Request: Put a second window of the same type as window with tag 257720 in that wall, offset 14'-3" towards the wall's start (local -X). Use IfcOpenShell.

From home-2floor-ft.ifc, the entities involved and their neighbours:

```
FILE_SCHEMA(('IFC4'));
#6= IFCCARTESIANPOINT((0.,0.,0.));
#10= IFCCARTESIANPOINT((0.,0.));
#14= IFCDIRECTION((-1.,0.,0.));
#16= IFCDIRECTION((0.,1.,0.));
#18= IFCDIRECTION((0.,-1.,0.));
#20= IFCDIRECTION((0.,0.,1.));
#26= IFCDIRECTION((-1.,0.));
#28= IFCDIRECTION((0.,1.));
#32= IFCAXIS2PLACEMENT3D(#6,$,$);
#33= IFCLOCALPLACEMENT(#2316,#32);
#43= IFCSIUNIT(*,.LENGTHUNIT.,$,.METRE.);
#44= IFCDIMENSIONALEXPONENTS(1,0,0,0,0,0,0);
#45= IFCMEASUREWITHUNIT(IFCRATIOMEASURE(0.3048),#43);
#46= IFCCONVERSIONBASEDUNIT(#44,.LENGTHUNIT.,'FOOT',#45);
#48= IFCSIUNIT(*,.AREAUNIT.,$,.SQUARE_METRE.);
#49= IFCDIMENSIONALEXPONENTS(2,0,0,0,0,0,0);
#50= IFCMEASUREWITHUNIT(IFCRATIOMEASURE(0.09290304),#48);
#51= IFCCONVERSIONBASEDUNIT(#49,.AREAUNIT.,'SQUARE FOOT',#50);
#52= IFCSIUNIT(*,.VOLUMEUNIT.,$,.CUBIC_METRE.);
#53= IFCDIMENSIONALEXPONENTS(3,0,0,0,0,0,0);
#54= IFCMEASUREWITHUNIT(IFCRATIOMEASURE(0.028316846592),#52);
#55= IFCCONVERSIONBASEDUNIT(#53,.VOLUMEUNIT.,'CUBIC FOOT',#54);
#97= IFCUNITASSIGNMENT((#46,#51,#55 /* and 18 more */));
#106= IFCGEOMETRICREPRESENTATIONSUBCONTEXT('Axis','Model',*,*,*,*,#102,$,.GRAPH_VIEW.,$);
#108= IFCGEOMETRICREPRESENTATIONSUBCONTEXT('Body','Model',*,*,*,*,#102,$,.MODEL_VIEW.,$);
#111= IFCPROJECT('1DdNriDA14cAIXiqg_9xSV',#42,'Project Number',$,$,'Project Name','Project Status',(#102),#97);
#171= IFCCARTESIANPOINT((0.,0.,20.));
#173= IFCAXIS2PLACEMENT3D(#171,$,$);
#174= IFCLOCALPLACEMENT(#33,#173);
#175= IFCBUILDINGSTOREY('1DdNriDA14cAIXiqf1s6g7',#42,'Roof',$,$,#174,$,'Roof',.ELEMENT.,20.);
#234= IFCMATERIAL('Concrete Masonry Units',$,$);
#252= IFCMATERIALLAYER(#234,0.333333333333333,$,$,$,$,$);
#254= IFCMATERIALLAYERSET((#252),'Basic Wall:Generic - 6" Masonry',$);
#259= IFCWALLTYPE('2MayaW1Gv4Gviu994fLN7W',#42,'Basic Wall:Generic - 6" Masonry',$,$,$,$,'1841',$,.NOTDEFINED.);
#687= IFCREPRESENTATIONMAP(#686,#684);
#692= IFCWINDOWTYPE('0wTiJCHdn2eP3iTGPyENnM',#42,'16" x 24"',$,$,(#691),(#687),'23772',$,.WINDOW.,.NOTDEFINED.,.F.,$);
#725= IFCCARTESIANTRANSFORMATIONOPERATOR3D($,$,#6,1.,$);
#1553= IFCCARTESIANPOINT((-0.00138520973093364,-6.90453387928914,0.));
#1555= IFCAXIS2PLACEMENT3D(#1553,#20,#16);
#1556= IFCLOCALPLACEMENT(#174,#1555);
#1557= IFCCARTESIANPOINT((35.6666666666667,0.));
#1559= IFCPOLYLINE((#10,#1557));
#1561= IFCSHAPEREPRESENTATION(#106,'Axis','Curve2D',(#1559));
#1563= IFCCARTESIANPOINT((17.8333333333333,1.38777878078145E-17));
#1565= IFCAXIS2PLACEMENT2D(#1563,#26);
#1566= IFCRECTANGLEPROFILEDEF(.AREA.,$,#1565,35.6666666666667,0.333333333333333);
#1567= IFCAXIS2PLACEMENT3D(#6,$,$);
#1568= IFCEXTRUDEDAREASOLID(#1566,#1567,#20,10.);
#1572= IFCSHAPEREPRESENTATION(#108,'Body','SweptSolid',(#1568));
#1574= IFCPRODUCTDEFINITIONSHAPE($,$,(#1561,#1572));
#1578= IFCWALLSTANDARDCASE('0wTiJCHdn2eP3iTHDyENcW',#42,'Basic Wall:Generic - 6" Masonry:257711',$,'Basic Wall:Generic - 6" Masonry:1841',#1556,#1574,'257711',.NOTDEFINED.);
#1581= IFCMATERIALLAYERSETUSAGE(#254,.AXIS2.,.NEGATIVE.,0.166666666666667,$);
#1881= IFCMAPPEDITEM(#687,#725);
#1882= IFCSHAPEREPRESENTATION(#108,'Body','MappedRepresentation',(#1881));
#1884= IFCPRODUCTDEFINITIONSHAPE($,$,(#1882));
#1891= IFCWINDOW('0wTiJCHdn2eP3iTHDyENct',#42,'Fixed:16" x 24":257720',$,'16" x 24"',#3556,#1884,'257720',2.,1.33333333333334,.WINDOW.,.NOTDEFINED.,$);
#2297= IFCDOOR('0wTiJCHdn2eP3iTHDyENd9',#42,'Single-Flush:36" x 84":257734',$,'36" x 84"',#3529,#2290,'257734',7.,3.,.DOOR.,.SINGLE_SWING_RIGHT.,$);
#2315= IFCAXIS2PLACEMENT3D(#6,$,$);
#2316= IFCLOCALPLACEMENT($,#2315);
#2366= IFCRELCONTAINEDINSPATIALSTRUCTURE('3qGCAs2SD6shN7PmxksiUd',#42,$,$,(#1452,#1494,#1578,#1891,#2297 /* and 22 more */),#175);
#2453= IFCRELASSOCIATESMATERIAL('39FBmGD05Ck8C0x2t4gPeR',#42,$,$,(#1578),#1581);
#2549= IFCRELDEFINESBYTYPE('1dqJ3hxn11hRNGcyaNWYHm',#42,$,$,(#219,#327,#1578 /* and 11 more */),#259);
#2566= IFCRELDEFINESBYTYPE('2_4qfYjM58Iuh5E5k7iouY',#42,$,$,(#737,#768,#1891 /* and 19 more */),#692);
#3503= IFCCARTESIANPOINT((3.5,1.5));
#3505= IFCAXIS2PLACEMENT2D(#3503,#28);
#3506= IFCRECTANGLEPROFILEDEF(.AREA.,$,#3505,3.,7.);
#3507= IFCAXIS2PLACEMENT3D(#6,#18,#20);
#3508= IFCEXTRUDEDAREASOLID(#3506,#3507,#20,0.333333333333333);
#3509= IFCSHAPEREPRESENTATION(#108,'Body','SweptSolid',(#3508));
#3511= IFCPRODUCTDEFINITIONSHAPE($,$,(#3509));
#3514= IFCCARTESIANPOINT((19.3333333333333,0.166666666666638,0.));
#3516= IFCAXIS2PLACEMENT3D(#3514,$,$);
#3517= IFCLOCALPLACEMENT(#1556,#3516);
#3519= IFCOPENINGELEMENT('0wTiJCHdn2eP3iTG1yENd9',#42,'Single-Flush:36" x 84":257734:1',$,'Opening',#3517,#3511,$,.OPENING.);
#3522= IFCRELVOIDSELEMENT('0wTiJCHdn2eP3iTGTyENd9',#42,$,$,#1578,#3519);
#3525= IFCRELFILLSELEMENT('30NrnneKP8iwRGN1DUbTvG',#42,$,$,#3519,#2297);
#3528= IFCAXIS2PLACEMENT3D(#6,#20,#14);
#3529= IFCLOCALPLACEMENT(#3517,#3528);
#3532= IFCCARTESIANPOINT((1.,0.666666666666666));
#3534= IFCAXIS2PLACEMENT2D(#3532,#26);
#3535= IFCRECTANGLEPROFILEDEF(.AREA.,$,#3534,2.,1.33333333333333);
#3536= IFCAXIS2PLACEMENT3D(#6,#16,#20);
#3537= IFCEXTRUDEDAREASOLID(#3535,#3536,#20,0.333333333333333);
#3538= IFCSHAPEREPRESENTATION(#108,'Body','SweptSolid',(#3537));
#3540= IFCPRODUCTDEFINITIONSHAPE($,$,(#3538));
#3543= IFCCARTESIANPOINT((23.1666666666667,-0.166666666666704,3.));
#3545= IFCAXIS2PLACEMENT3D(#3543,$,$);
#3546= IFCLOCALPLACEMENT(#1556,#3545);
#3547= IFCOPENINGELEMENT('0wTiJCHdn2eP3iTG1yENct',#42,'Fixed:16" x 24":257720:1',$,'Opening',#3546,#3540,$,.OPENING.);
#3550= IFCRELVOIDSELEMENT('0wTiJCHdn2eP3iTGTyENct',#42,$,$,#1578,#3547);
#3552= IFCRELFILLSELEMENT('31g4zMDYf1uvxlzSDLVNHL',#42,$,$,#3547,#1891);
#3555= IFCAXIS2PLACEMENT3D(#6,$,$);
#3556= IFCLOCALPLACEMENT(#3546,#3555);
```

```python
import ifcopenshell
import ifcopenshell.api.feature
import ifcopenshell.api.geometry
import ifcopenshell.api.root
import ifcopenshell.geom
import ifcopenshell.util.element
import ifcopenshell.util.placement
import ifcopenshell.util.shape
import ifcopenshell.util.unit

model = ifcopenshell.open("home-2floor-ft.ifc")
unit_scale = ifcopenshell.util.unit.calculate_unit_scale(model)
settings = ifcopenshell.geom.settings()


def volume(element):
    """Net volume in cubic metres, openings subtracted."""
    shape = ifcopenshell.geom.create_shape(settings, element)
    return ifcopenshell.util.shape.get_volume(shape.geometry)


def reuse_history(source, copy):
    """copy_class also copies each property set's owner history, people and application; keep the originals."""
    for rel in copy.IsDefinedBy:
        if rel.is_a("IfcRelDefinesByProperties") and (history := rel.RelatingPropertyDefinition.OwnerHistory):
            rel.RelatingPropertyDefinition.OwnerHistory = source.OwnerHistory
            ifcopenshell.util.element.remove_deep2(model, history)


window = model.by_id(1891)
opening = window.FillsVoids[0].RelatingOpeningElement
wall = opening.VoidsElements[0].RelatingBuildingElement
before = volume(wall)
shift = ifcopenshell.util.placement.get_local_placement(wall.ObjectPlacement)[:3, 0] * -171 * 0.0254 / unit_scale

# copy_class copies the void relationship, type, container and properties, but no geometry.
new_opening = ifcopenshell.api.root.copy_class(model, product=opening)
new_opening.Representation = ifcopenshell.util.element.copy_deep(
    model, opening.Representation, exclude=["IfcGeometricRepresentationContext", "IfcRepresentationMap"]
)
new_opening.Name = 'Fixed:16" x 24"'
new_window = ifcopenshell.api.root.copy_class(model, product=window)
new_window.Representation = ifcopenshell.util.element.copy_deep(
    model, window.Representation, exclude=["IfcGeometricRepresentationContext", "IfcRepresentationMap"]
)
new_window.Name = 'Fixed:16" x 24"'
new_window.Tag = None
reuse_history(window, new_window)
ifcopenshell.api.feature.add_filling(model, opening=new_opening, element=new_window)

for old, new in ((opening, new_opening), (window, new_window)):
    matrix = ifcopenshell.util.placement.get_local_placement(old.ObjectPlacement)
    matrix[:3, 3] += shift
    ifcopenshell.api.geometry.edit_object_placement(model, product=new, matrix=matrix, is_si=False)

after = volume(wall)

print(f"wall volume {before:.3f} -> {after:.3f} m3")

model.write("home-2floor-ft_updated.ifc")
```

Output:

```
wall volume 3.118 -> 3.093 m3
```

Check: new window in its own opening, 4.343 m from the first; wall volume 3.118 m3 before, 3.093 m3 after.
